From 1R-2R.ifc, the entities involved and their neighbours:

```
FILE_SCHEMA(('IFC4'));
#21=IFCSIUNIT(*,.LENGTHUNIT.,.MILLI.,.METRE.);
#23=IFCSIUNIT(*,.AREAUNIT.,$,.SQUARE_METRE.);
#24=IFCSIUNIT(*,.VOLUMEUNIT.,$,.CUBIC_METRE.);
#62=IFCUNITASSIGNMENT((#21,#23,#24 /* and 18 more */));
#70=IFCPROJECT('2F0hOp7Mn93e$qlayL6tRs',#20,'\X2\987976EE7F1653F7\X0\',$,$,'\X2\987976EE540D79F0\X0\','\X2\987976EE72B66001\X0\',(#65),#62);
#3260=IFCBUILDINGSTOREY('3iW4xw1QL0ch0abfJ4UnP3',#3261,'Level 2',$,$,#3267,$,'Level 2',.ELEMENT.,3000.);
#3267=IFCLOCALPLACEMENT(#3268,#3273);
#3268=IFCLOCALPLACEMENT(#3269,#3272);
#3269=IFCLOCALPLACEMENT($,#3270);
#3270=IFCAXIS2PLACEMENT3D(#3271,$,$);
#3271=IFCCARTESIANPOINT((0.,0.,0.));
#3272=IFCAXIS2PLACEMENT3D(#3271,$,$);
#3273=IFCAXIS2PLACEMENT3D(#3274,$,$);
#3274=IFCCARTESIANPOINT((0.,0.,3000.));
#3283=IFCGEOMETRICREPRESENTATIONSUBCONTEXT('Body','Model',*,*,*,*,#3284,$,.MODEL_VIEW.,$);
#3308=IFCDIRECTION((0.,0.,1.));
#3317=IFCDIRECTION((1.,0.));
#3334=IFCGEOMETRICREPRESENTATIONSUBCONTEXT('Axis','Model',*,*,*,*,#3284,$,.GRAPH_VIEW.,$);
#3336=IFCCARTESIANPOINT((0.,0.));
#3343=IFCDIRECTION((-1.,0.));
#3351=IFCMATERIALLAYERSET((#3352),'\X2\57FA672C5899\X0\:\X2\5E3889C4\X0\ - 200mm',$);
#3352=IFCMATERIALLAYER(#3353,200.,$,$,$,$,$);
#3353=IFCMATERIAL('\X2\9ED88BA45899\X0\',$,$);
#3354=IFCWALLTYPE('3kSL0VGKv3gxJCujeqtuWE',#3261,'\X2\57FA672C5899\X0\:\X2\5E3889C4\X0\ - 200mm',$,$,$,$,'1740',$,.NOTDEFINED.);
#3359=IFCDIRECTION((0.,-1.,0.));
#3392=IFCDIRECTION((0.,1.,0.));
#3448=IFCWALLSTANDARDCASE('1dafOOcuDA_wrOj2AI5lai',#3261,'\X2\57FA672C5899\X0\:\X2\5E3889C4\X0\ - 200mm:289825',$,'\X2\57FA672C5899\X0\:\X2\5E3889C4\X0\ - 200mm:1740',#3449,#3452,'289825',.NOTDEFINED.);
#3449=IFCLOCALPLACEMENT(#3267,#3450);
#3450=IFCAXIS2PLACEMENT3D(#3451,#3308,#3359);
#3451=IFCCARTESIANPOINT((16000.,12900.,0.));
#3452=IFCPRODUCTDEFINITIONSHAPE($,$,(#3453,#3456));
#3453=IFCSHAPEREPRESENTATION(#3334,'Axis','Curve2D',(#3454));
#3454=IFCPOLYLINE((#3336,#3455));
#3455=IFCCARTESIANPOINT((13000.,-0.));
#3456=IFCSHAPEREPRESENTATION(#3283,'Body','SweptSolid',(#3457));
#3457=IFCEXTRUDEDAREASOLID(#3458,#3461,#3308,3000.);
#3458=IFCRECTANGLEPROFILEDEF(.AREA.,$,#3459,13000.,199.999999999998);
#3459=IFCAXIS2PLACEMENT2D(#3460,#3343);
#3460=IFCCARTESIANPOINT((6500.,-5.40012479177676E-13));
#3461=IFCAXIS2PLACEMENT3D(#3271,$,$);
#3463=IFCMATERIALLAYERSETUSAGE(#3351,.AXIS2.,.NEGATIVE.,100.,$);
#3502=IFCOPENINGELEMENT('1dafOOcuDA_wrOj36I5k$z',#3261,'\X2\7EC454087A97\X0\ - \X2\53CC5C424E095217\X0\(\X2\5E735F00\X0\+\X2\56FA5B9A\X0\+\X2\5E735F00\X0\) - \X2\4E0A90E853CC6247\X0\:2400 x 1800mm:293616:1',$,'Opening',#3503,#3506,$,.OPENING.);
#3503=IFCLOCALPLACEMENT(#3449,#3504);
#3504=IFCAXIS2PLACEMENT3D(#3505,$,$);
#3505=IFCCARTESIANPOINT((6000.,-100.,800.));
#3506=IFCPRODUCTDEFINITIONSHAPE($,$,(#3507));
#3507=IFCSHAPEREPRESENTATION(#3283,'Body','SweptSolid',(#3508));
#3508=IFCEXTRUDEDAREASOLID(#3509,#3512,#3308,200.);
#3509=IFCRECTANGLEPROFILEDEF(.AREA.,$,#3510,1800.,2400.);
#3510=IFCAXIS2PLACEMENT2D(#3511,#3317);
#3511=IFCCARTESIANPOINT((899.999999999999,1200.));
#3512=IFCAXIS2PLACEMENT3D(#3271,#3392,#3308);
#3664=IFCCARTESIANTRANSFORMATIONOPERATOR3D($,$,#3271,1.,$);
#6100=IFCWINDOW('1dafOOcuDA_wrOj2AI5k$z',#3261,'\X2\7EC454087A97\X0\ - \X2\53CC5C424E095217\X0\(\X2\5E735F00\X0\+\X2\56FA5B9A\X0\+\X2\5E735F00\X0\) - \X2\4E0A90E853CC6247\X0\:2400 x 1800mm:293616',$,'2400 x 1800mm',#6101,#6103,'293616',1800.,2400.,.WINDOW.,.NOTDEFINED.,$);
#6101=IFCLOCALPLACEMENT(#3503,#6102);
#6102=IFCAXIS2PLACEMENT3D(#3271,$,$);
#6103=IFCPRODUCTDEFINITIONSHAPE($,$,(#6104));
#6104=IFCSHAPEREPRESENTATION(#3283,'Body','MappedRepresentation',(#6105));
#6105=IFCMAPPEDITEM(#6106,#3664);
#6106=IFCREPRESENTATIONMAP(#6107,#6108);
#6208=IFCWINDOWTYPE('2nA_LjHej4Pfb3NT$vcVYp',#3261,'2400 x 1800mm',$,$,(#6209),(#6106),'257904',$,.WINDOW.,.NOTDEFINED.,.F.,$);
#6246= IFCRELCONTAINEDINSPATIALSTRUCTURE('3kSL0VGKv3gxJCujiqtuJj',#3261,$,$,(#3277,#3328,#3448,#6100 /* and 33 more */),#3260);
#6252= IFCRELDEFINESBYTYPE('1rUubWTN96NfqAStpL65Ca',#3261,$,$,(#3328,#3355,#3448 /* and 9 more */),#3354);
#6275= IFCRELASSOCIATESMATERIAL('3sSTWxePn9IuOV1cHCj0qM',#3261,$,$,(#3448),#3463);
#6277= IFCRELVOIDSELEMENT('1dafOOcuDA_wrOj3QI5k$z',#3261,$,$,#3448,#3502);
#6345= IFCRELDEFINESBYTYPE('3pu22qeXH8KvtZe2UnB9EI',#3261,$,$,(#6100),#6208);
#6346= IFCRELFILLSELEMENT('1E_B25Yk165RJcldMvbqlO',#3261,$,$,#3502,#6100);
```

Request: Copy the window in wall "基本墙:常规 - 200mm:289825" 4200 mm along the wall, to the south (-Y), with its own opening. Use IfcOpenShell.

```python
import ifcopenshell
import ifcopenshell.api.feature
import ifcopenshell.api.geometry
import ifcopenshell.api.root
import ifcopenshell.geom
import ifcopenshell.util.element
import ifcopenshell.util.placement
import ifcopenshell.util.shape
import ifcopenshell.util.unit

model = ifcopenshell.open("1R-2R.ifc")
unit_scale = ifcopenshell.util.unit.calculate_unit_scale(model)
settings = ifcopenshell.geom.settings()


def volume(element):
    """Net volume in cubic metres, openings subtracted."""
    shape = ifcopenshell.geom.create_shape(settings, element)
    return ifcopenshell.util.shape.get_volume(shape.geometry)


def reuse_history(source, copy):
    """copy_class also copies each property set's owner history, people and application; keep the originals."""
    for rel in copy.IsDefinedBy:
        if rel.is_a("IfcRelDefinesByProperties") and (history := rel.RelatingPropertyDefinition.OwnerHistory):
            rel.RelatingPropertyDefinition.OwnerHistory = source.OwnerHistory
            ifcopenshell.util.element.remove_deep2(model, history)


window = model.by_id(6100)
opening = window.FillsVoids[0].RelatingOpeningElement
wall = opening.VoidsElements[0].RelatingBuildingElement
before = volume(wall)
shift = ifcopenshell.util.placement.get_local_placement(wall.ObjectPlacement)[:3, 0] * 4.2 / unit_scale

# copy_class copies the void relationship, type, container and properties, but no geometry.
new_opening = ifcopenshell.api.root.copy_class(model, product=opening)
new_opening.Representation = ifcopenshell.util.element.copy_deep(
    model, opening.Representation, exclude=["IfcGeometricRepresentationContext", "IfcRepresentationMap"]
)
new_opening.Name = "组合窗 - 双层三列(平开+固定+平开) - 上部双扇:2400 x 1800mm"
new_window = ifcopenshell.api.root.copy_class(model, product=window)
new_window.Representation = ifcopenshell.util.element.copy_deep(
    model, window.Representation, exclude=["IfcGeometricRepresentationContext", "IfcRepresentationMap"]
)
new_window.Name = "组合窗 - 双层三列(平开+固定+平开) - 上部双扇:2400 x 1800mm"
new_window.Tag = None
reuse_history(window, new_window)
ifcopenshell.api.feature.add_filling(model, opening=new_opening, element=new_window)

for old, new in ((opening, new_opening), (window, new_window)):
    matrix = ifcopenshell.util.placement.get_local_placement(old.ObjectPlacement)
    matrix[:3, 3] += shift
    ifcopenshell.api.geometry.edit_object_placement(model, product=new, matrix=matrix, is_si=False)

after = volume(wall)

print(f"wall volume {before:.3f} -> {after:.3f} m3")

model.write("1R-2R_edited.ifc")
```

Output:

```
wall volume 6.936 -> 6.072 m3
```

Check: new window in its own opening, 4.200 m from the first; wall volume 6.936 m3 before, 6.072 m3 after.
